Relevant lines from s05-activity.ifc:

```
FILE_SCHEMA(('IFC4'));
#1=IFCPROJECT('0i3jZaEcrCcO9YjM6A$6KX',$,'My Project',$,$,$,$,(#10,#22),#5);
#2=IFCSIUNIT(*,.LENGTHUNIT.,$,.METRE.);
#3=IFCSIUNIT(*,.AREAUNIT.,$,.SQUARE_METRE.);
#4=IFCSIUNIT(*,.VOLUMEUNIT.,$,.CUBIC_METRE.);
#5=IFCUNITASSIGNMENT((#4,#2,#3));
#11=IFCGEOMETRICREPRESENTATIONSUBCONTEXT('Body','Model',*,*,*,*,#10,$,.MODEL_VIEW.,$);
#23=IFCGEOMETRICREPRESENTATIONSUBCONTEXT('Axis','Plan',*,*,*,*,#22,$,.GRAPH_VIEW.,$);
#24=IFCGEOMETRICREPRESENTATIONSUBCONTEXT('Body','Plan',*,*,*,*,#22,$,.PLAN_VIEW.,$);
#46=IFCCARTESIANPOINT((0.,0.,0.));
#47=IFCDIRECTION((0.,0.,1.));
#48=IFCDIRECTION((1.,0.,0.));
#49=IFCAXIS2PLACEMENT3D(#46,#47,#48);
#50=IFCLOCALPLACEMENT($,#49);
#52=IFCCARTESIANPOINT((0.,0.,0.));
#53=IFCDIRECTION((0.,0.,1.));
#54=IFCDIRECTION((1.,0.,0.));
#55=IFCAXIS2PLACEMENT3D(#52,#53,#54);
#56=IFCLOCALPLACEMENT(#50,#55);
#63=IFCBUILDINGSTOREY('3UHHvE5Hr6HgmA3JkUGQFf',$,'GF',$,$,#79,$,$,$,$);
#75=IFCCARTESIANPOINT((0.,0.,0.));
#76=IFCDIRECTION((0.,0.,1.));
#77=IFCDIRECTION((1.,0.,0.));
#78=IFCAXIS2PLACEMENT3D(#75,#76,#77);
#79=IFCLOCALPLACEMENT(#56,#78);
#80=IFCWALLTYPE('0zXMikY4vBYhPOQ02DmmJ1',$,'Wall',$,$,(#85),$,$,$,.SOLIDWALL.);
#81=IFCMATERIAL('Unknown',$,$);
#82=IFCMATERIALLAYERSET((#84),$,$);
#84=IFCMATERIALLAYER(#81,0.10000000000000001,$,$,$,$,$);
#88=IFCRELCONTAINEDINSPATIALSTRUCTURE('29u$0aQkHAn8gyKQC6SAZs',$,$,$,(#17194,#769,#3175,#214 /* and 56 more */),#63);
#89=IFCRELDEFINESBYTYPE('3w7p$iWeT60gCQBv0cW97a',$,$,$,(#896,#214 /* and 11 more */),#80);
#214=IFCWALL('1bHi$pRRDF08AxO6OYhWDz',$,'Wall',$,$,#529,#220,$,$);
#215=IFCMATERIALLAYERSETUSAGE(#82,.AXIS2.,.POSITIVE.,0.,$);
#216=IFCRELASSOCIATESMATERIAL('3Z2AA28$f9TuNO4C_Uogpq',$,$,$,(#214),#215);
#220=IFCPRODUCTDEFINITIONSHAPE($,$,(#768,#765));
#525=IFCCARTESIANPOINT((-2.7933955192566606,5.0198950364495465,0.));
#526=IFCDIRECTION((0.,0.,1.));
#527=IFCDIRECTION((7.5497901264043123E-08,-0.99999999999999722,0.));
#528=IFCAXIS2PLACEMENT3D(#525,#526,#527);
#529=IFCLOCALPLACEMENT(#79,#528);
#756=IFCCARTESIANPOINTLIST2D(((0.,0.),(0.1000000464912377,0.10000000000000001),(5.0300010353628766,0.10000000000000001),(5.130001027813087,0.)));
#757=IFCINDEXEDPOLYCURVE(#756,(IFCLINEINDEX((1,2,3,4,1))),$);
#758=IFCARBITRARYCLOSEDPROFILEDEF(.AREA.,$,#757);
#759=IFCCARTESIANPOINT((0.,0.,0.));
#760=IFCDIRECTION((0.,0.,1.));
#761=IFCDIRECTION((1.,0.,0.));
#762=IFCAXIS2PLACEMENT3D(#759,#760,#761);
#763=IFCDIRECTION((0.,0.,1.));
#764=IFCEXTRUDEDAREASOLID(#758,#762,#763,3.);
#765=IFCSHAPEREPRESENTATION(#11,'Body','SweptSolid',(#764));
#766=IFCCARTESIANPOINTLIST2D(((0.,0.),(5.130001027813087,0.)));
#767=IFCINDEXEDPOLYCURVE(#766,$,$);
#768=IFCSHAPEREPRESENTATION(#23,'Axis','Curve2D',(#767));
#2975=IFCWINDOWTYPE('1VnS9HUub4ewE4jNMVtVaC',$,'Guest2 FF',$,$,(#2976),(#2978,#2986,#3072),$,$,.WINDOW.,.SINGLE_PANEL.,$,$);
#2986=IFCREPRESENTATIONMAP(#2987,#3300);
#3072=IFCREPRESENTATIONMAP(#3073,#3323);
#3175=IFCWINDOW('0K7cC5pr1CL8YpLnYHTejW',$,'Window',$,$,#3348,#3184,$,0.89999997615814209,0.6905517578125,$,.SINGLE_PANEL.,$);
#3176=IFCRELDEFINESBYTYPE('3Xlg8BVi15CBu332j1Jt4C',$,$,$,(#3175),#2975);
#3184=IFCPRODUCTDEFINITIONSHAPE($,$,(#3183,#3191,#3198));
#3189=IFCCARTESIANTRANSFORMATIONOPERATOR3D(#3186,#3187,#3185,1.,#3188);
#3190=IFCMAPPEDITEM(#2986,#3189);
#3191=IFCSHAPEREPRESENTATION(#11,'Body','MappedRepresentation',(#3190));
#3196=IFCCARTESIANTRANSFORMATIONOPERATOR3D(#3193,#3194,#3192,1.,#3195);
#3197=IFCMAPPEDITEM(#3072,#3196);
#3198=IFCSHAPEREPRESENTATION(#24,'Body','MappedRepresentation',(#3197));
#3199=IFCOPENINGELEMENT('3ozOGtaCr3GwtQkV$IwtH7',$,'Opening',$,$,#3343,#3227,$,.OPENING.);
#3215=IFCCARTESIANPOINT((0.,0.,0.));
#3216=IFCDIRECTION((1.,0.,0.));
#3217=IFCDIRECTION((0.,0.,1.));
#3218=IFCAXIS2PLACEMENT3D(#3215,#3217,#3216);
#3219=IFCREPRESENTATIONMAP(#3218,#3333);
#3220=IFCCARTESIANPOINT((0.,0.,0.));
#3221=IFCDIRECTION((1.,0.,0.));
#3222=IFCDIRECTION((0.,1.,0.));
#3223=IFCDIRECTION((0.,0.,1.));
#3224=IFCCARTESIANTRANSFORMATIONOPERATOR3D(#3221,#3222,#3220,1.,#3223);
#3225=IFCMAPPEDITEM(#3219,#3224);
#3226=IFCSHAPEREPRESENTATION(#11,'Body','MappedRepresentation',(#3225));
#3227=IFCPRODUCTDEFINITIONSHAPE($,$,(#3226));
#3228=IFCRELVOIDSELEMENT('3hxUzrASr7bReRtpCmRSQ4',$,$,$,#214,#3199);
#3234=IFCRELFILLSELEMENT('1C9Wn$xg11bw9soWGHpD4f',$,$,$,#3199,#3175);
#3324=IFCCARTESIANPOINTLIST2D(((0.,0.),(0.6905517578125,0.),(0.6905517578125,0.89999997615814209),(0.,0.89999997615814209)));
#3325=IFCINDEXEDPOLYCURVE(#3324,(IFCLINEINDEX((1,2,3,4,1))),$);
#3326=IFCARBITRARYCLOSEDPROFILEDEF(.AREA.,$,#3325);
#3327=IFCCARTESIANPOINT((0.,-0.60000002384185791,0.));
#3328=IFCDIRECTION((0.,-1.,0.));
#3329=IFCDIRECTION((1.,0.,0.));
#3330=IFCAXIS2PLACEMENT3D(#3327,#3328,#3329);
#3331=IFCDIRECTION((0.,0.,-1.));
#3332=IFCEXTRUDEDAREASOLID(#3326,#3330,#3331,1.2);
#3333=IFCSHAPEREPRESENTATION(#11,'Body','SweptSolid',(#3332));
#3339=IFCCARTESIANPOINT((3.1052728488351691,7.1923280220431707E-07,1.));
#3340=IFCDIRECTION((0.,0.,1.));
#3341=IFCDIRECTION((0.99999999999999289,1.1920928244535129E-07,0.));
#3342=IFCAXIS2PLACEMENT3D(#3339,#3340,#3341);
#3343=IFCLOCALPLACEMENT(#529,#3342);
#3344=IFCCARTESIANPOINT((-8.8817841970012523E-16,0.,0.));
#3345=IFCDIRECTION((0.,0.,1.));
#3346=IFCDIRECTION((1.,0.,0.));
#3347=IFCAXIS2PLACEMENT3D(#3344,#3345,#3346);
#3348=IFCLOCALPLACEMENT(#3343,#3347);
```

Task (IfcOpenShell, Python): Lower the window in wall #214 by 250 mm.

```python
import numpy as np
import ifcopenshell
import ifcopenshell.api.geometry
import ifcopenshell.util.placement
import ifcopenshell.util.unit

model = ifcopenshell.open("s05-activity.ifc")
unit_scale = ifcopenshell.util.unit.calculate_unit_scale(model)

window = model.by_guid("0K7cC5pr1CL8YpLnYHTejW")
opening = window.FillsVoids[0].RelatingOpeningElement
dz = -0.25 / unit_scale

shift = np.array([0.0, 0.0, dz])
# The window is placed relative to its opening, so it follows when the opening moves.
matrix = ifcopenshell.util.placement.get_local_placement(opening.ObjectPlacement)
matrix[:3, 3] += shift
ifcopenshell.api.geometry.edit_object_placement(
    model, product=opening, matrix=matrix, is_si=False, should_transform_children=True
)

print(f"moved by {dz * unit_scale:+.3f} m")

model.write("s05-activity_v2.ifc")
```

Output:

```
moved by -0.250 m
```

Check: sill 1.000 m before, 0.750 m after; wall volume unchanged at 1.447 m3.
